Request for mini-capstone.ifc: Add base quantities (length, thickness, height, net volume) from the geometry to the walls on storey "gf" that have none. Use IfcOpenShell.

First a look at what the model holds.

```python
import ifcopenshell
import ifcopenshell.util.element
import ifcopenshell.util.unit

model = ifcopenshell.open("mini-capstone.ifc")
print(model.schema)
for unit_type in ("LENGTHUNIT", "AREAUNIT", "VOLUMEUNIT"):
    print(unit_type, ifcopenshell.util.unit.calculate_unit_scale(model, unit_type))
storey = next(s for s in model.by_type("IfcBuildingStorey") if s.Name == "gf")
walls = [e for e in ifcopenshell.util.element.get_decomposition(storey) if e.is_a("IfcWall")]
for e in sorted(walls, key=lambda e: e.id()):
    print(e.id(), e.is_a(), e.Name, list(ifcopenshell.util.element.get_psets(e, qtos_only=True)), sep=" | ")
```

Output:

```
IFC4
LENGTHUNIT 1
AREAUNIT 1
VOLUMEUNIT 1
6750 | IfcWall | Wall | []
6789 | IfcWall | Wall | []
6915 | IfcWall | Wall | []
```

```python
import ifcopenshell
import ifcopenshell.api.pset
import ifcopenshell.geom
import ifcopenshell.util.element
import ifcopenshell.util.shape
import ifcopenshell.util.unit

model = ifcopenshell.open("mini-capstone.ifc")
unit_scale = ifcopenshell.util.unit.calculate_unit_scale(model)
volume_scale = ifcopenshell.util.unit.calculate_unit_scale(model, "VOLUMEUNIT")
settings = ifcopenshell.geom.settings()

storey = next(s for s in model.by_type("IfcBuildingStorey") if s.Name == "gf")
walls = [e for e in ifcopenshell.util.element.get_decomposition(storey) if e.is_a("IfcWall")]

for e in sorted(walls, key=lambda e: e.id()):
    if ifcopenshell.util.element.get_psets(e, qtos_only=True, should_inherit=False):
        continue
    # Geometry comes back in metres, in the element's own axes.
    shape = ifcopenshell.geom.create_shape(settings, e)
    values = {
        "Length": ifcopenshell.util.shape.get_x(shape.geometry) / unit_scale,
        "Width": ifcopenshell.util.shape.get_y(shape.geometry) / unit_scale,
        "Height": ifcopenshell.util.shape.get_z(shape.geometry) / unit_scale,
        "NetVolume": ifcopenshell.util.shape.get_volume(shape.geometry) / volume_scale,
    }
    qto = ifcopenshell.api.pset.add_qto(model, product=e, name="Qto_WallBaseQuantities")
    ifcopenshell.api.pset.edit_qto(model, qto=qto, properties=values)
    print(e.id(), {k: round(v, 3) for k, v in values.items()})

model.write("mini-capstone_v2.ifc")
```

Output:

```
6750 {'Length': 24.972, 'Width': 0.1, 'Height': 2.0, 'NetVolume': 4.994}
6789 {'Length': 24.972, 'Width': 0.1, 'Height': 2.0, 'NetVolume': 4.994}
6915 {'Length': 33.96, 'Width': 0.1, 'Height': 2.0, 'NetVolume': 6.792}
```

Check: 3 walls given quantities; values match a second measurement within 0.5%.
